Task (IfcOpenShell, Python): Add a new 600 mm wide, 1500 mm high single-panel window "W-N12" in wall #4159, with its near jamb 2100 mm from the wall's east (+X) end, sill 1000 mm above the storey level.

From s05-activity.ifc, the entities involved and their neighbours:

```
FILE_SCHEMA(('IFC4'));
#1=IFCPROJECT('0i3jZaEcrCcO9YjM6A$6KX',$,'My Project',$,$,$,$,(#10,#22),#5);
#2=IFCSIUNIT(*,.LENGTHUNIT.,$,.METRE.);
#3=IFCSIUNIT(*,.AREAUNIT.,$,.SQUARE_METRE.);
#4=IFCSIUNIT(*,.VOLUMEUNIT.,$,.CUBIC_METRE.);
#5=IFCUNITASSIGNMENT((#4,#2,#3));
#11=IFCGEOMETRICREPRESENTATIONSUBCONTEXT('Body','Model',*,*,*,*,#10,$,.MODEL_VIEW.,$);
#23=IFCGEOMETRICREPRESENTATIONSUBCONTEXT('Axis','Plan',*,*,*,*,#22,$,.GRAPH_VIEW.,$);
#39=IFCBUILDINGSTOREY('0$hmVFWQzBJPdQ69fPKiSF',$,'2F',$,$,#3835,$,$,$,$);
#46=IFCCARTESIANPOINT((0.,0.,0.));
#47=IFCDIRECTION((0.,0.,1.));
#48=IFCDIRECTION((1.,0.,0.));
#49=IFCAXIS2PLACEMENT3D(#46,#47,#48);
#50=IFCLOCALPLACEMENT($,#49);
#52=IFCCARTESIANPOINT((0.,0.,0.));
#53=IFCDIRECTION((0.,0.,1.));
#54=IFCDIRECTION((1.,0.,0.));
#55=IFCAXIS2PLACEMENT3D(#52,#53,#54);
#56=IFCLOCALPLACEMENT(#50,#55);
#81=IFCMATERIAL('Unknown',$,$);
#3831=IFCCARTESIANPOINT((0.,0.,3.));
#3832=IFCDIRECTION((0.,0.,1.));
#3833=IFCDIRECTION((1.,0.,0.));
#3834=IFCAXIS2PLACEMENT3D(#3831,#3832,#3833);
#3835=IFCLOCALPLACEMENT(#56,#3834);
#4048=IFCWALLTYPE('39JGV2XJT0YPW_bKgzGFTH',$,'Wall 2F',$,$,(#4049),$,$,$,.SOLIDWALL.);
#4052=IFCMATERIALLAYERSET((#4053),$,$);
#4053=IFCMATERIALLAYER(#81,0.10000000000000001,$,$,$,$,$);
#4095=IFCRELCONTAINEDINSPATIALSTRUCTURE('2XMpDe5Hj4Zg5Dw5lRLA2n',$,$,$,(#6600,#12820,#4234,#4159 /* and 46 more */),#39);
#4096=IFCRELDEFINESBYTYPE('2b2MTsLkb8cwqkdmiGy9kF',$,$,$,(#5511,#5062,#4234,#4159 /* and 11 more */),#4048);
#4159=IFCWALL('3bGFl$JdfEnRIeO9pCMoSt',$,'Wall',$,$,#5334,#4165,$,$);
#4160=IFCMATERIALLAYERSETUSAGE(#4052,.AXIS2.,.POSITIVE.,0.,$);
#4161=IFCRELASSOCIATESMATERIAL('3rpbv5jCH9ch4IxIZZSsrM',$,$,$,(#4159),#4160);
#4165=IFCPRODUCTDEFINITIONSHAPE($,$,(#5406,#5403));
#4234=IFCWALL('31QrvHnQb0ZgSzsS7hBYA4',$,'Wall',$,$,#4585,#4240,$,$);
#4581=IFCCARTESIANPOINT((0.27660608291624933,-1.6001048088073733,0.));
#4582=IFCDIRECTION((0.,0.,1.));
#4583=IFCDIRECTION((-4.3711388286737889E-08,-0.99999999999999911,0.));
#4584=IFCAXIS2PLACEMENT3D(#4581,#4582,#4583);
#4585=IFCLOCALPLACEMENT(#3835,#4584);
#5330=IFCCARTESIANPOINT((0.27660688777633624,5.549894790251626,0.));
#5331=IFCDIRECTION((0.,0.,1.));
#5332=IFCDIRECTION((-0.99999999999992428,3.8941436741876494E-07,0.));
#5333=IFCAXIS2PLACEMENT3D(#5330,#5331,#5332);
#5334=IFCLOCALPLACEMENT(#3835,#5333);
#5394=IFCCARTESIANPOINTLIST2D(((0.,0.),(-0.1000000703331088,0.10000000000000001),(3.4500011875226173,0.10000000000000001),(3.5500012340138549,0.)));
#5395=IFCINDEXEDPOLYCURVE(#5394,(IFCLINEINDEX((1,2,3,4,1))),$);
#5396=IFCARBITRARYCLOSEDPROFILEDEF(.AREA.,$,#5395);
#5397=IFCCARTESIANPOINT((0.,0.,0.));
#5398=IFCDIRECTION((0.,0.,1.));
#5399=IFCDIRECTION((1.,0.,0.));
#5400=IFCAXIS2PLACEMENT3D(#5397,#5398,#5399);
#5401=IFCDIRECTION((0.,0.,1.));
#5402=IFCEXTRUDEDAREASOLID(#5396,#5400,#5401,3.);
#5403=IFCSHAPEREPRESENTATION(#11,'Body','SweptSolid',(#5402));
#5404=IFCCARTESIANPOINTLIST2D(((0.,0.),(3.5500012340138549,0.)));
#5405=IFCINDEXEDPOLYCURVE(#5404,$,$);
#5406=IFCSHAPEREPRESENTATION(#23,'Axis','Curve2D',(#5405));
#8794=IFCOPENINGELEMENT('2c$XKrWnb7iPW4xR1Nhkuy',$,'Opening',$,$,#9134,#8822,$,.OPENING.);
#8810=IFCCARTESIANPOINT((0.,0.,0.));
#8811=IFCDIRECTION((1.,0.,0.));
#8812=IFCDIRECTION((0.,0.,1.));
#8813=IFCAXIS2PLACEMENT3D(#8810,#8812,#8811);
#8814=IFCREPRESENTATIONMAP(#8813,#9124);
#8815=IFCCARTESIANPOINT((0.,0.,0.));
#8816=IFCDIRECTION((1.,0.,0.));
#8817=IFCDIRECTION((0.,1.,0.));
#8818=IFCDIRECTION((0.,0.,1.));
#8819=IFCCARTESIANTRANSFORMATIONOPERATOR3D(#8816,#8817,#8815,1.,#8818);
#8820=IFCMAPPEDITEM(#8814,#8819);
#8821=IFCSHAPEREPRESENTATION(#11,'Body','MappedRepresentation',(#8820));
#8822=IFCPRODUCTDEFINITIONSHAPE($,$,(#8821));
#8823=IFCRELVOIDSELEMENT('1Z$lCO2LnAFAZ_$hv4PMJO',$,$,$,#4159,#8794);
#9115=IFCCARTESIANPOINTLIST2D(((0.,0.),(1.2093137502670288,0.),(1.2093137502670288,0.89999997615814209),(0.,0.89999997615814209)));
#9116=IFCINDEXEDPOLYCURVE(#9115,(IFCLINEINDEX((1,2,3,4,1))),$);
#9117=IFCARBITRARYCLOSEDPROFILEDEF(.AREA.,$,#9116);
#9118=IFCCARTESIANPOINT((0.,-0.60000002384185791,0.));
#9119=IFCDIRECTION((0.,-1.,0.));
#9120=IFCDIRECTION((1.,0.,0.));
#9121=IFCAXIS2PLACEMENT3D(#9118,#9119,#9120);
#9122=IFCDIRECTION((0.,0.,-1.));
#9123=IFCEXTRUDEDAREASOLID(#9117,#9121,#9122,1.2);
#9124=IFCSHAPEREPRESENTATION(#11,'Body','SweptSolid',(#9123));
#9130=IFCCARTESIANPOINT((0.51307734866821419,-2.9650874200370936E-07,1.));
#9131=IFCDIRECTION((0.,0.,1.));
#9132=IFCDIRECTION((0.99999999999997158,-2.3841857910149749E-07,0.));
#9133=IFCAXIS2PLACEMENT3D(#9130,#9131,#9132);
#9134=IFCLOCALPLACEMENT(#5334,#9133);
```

```python
import numpy as np
import ifcopenshell
import ifcopenshell.api.feature
import ifcopenshell.api.geometry
import ifcopenshell.api.root
import ifcopenshell.api.spatial
import ifcopenshell.geom
import ifcopenshell.util.element
import ifcopenshell.util.placement
import ifcopenshell.util.representation
import ifcopenshell.util.shape
import ifcopenshell.util.unit

model = ifcopenshell.open("s05-activity.ifc")
unit_scale = ifcopenshell.util.unit.calculate_unit_scale(model)
settings = ifcopenshell.geom.settings()


def volume(element):
    """Net volume in cubic metres, openings subtracted."""
    shape = ifcopenshell.geom.create_shape(settings, element)
    return ifcopenshell.util.shape.get_volume(shape.geometry)


wall = model.by_id(4159)
storey = ifcopenshell.util.element.get_container(wall, ifc_class="IfcBuildingStorey")
context = ifcopenshell.util.representation.get_context(model, "Model", "Body", "MODEL_VIEW")
before = volume(wall)

width, height, from_end, sill = 0.6, 1.5, 2.1, 1  # metres

# The wall runs along its own X axis, and the end named is its -X end.
wall_shape = ifcopenshell.geom.create_shape(settings, wall)
x, y, z = ifcopenshell.util.shape.get_vertices(wall_shape.geometry).T
start = x.min() + from_end
face, thickness = float(y.min()), float(y.max() - y.min())
wall_matrix = ifcopenshell.util.placement.get_local_placement(wall.ObjectPlacement)
level = ifcopenshell.util.placement.get_local_placement(storey.ObjectPlacement)[2, 3]


def in_wall(x, y):
    """Placement at x, y metres in the wall's axes, at sill height."""
    matrix = wall_matrix.copy()
    matrix[:, 3] = wall_matrix @ np.array([x / unit_scale, y / unit_scale, 0.0, 1.0])
    matrix[2, 3] = level + sill / unit_scale
    return matrix


# Opening: a box that overshoots both wall faces by 50 mm.
opening = ifcopenshell.api.root.create_entity(model, ifc_class="IfcOpeningElement", predefined_type="OPENING")
box = ifcopenshell.api.geometry.add_wall_representation(
    model, context=context, length=width, height=height, thickness=thickness + 0.1
)
ifcopenshell.api.geometry.assign_representation(model, product=opening, representation=box)
ifcopenshell.api.geometry.edit_object_placement(model, product=opening, matrix=in_wall(start, face - 0.05), is_si=False)
ifcopenshell.api.feature.add_feature(model, feature=opening, element=wall)

window = ifcopenshell.api.root.create_entity(model, ifc_class="IfcWindow", name="W-N12", predefined_type="WINDOW")
window.OverallWidth, window.OverallHeight = width / unit_scale, height / unit_scale
window.PartitioningType = "SINGLE_PANEL"
body = ifcopenshell.api.geometry.add_window_representation(
    model,
    context=context,
    overall_width=window.OverallWidth,
    overall_height=window.OverallHeight,
    partition_type="SINGLE_PANEL",
)
ifcopenshell.api.geometry.assign_representation(model, product=window, representation=body)
ifcopenshell.api.spatial.assign_container(model, products=[window], relating_structure=storey)
ifcopenshell.api.feature.add_filling(model, opening=opening, element=window)

# Centre the window in the wall's thickness.
ifcopenshell.api.geometry.edit_object_placement(model, product=window, matrix=in_wall(start, face), is_si=False)
window_shape = ifcopenshell.geom.create_shape(settings, window)
depth = ifcopenshell.util.shape.get_vertices(window_shape.geometry)[:, 1]
offset = face + thickness / 2 - (depth.min() + depth.max()) / 2
ifcopenshell.api.geometry.edit_object_placement(model, product=window, matrix=in_wall(start, offset), is_si=False)

after = volume(wall)

print(f"wall volume {before:.3f} -> {after:.3f} m3")

model.write("s05-activity_edited.ifc")
```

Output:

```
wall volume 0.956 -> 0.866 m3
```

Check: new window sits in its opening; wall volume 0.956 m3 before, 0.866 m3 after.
